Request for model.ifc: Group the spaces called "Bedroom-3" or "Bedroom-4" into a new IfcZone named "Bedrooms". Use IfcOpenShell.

First a look at what the model holds.

```python
import ifcopenshell

model = ifcopenshell.open("model.ifc")
print(model.schema)
seen = {}
for space in model.by_type("IfcSpace"):
    seen[space.Name] = seen.get(space.Name, 0) + 1
for name, count in sorted(seen.items(), key=str):
    print(count, "x", name)
print("zones:", [z.Name for z in model.by_type("IfcZone")][:20])
```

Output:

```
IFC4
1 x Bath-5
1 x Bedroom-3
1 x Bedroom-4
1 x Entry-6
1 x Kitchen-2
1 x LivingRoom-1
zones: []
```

```python
import ifcopenshell
import ifcopenshell.api.group
import ifcopenshell.api.root

model = ifcopenshell.open("model.ifc")

names = {"Bedroom-3", "Bedroom-4"}
spaces = [s for s in model.by_type("IfcSpace") if s.Name in names]

zone = ifcopenshell.api.root.create_entity(model, ifc_class="IfcZone", name="Bedrooms")
ifcopenshell.api.group.assign_group(model, products=spaces, group=zone)
print(len(spaces), "spaces in", zone.Name)

model.write("model_edited.ifc")
```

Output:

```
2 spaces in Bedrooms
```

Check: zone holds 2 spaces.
